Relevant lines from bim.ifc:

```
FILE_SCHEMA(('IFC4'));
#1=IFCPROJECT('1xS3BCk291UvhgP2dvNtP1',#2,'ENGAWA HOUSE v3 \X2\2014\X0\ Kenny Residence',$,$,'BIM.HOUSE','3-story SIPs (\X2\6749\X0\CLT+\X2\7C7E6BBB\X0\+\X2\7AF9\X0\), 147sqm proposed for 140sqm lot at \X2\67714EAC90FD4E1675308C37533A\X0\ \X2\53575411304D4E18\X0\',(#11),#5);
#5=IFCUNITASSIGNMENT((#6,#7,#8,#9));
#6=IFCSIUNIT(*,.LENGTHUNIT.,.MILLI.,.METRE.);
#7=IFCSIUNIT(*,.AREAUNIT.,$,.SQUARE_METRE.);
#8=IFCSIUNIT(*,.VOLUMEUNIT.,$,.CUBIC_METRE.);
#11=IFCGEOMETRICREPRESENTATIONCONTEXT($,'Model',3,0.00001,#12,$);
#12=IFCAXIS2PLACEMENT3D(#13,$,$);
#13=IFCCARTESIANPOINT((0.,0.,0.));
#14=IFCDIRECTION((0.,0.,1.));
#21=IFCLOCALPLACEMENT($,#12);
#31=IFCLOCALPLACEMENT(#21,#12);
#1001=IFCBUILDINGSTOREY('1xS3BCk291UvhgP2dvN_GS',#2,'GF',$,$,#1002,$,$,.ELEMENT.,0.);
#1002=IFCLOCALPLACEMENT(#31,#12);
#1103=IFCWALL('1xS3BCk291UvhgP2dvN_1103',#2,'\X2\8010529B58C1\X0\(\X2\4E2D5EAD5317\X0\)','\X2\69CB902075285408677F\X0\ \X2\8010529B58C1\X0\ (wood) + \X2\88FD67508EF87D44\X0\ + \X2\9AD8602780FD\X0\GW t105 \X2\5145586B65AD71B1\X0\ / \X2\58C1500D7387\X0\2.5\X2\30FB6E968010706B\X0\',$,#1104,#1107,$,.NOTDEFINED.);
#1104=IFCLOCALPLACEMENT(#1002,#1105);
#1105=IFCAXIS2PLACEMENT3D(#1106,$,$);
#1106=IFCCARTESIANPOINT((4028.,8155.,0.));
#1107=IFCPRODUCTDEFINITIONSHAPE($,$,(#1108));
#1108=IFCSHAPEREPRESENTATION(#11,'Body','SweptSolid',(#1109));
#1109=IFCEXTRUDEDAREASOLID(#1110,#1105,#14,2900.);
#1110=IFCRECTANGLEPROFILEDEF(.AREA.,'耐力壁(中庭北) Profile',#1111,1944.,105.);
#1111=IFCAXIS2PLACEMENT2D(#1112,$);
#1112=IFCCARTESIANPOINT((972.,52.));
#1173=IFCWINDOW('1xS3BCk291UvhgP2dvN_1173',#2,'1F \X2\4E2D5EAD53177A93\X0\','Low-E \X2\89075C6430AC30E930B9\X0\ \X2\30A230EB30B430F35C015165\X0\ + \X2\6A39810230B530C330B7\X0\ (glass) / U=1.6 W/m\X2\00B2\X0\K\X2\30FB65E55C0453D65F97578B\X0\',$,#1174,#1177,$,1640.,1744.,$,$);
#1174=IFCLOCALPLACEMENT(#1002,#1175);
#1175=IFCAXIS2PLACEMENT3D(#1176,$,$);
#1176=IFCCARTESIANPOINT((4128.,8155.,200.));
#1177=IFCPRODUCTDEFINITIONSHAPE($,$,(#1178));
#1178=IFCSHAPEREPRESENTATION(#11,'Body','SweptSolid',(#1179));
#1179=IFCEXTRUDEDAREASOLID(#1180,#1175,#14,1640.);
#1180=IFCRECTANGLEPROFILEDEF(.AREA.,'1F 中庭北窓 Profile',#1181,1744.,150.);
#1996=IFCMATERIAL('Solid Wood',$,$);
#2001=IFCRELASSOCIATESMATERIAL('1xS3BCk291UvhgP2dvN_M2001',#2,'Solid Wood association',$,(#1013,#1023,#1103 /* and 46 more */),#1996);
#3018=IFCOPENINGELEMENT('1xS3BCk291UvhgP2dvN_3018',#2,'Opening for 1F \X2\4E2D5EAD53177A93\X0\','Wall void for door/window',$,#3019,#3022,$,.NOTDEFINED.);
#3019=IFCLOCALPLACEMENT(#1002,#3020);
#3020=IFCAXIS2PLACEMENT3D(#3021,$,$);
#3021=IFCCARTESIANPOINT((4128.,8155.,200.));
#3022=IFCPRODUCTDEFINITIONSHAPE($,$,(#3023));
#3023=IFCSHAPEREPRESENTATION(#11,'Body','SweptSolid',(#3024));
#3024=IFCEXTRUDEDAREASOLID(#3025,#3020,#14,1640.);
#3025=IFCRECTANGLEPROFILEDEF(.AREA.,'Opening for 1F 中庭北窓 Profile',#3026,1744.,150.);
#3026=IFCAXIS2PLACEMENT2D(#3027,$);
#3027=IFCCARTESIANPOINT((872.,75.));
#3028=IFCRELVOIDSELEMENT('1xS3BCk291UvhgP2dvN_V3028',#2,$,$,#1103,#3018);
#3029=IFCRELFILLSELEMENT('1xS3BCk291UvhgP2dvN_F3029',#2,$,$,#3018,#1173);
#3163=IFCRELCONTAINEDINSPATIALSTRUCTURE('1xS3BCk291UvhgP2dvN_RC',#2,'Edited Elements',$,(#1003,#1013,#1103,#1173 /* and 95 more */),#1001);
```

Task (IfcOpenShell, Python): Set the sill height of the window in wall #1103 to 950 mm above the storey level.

```python
import numpy as np
import ifcopenshell
import ifcopenshell.api.geometry
import ifcopenshell.geom
import ifcopenshell.util.element
import ifcopenshell.util.placement
import ifcopenshell.util.shape
import ifcopenshell.util.unit

model = ifcopenshell.open("bim.ifc")
unit_scale = ifcopenshell.util.unit.calculate_unit_scale(model)

window = model.by_guid("1xS3BCk291UvhgP2dvN_1173")
opening = window.FillsVoids[0].RelatingOpeningElement
storey = ifcopenshell.util.element.get_container(window, ifc_class="IfcBuildingStorey")
level = ifcopenshell.util.placement.get_local_placement(storey.ObjectPlacement)[2, 3]

# The opening's origin need not be at the sill, so measure its lowest point.
shape = ifcopenshell.geom.create_shape(ifcopenshell.geom.settings(), opening)
bottom = ifcopenshell.util.shape.get_shape_bottom_elevation(shape, shape.geometry) / unit_scale
dz = level + 950.0 - bottom

shift = np.array([0.0, 0.0, dz])
# The window is not placed relative to its opening, so move both.
for product in (opening, window):
    matrix = ifcopenshell.util.placement.get_local_placement(product.ObjectPlacement)
    matrix[:3, 3] += shift
    ifcopenshell.api.geometry.edit_object_placement(model, product=product, matrix=matrix, is_si=False)

print(f"moved by {dz * unit_scale:+.3f} m")

model.write("bim_updated.ifc")
```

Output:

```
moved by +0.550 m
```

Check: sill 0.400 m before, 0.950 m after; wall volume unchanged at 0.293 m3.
